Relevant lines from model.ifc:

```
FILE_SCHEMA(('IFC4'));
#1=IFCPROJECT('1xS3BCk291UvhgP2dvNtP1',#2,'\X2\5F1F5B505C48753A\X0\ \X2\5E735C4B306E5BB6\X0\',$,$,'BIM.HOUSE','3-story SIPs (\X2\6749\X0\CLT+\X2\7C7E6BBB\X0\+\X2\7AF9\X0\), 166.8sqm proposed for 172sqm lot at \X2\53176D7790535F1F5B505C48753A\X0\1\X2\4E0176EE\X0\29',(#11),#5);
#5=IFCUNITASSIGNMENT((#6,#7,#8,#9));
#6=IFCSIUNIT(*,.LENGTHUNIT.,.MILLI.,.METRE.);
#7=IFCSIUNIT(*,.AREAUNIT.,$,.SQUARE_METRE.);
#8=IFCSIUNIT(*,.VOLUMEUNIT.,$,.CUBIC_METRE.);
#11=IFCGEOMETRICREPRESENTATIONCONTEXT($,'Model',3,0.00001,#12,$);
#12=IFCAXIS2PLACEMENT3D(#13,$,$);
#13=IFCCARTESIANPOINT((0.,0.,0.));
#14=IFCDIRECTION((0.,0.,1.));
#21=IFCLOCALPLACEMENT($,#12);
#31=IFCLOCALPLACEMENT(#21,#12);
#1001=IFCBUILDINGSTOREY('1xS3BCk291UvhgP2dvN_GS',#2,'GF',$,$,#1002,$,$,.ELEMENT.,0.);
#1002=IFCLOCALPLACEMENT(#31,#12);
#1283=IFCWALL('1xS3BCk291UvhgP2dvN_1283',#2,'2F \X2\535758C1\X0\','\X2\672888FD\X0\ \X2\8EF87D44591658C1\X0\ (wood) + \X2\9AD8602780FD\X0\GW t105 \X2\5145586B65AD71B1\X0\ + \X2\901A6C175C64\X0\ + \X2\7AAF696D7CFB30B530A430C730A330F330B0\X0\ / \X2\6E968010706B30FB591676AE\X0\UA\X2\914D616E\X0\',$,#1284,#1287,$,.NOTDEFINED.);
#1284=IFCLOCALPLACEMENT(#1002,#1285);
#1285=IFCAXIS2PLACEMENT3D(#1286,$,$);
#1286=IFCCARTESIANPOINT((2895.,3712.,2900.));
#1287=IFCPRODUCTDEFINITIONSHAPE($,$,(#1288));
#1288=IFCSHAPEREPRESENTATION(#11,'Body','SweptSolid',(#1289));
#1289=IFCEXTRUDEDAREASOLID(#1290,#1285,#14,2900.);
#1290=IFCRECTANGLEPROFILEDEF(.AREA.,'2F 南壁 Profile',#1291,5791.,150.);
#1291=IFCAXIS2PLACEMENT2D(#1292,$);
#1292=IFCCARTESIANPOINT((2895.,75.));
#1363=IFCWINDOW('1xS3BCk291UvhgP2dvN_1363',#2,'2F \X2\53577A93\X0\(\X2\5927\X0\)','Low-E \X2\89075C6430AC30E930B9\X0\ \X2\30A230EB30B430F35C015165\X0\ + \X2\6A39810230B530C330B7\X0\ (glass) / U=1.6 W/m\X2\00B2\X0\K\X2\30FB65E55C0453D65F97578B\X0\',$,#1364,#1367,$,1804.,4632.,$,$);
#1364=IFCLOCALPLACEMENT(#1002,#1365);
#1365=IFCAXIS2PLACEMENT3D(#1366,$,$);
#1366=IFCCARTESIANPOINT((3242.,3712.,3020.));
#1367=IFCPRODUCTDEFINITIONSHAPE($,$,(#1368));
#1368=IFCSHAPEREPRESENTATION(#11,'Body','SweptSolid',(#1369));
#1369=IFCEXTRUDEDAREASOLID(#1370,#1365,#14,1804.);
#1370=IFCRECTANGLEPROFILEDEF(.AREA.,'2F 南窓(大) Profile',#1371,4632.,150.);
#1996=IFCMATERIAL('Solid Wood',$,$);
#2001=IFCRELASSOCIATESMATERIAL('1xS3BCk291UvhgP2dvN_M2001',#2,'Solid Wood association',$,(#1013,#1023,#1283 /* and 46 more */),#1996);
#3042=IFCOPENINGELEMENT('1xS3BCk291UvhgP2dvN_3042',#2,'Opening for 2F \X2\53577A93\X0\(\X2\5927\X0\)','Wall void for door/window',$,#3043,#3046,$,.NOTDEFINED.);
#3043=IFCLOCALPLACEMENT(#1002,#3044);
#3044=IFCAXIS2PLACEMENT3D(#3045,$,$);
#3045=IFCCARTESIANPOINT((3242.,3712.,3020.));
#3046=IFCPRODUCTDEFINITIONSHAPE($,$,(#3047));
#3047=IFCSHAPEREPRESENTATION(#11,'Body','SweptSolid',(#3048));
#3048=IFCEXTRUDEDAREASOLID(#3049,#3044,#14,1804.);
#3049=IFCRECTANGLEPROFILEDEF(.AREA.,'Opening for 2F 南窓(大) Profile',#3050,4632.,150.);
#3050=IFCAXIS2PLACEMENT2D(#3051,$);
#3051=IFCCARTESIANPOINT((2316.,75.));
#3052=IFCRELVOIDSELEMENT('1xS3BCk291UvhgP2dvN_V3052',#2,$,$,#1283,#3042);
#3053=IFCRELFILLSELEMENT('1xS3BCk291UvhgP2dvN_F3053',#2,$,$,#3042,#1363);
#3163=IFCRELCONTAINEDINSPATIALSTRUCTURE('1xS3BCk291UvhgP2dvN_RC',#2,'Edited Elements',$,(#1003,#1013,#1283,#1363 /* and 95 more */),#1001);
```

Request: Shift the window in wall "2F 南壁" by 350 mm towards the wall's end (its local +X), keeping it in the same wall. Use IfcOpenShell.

```python
import ifcopenshell
import ifcopenshell.api.geometry
import ifcopenshell.util.placement
import ifcopenshell.util.unit

model = ifcopenshell.open("model.ifc")
unit_scale = ifcopenshell.util.unit.calculate_unit_scale(model)

window = model.by_guid("1xS3BCk291UvhgP2dvN_1363")
opening = window.FillsVoids[0].RelatingOpeningElement
wall = opening.VoidsElements[0].RelatingBuildingElement

wall_matrix = ifcopenshell.util.placement.get_local_placement(wall.ObjectPlacement)
shift = wall_matrix[:3, 0] * 0.35 / unit_scale
before = ifcopenshell.util.placement.get_local_placement(window.ObjectPlacement)[:3, 3].copy()

# The window is not placed relative to its opening, so move both.
for product in (opening, window):
    matrix = ifcopenshell.util.placement.get_local_placement(product.ObjectPlacement)
    matrix[:3, 3] += shift
    ifcopenshell.api.geometry.edit_object_placement(model, product=product, matrix=matrix, is_si=False)

after = ifcopenshell.util.placement.get_local_placement(window.ObjectPlacement)[:3, 3]
print("window moved by", (after - before).round(3) + 0.0)

model.write("model-out.ifc")
```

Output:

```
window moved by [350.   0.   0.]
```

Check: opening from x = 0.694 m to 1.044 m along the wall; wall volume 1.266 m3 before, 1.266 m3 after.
